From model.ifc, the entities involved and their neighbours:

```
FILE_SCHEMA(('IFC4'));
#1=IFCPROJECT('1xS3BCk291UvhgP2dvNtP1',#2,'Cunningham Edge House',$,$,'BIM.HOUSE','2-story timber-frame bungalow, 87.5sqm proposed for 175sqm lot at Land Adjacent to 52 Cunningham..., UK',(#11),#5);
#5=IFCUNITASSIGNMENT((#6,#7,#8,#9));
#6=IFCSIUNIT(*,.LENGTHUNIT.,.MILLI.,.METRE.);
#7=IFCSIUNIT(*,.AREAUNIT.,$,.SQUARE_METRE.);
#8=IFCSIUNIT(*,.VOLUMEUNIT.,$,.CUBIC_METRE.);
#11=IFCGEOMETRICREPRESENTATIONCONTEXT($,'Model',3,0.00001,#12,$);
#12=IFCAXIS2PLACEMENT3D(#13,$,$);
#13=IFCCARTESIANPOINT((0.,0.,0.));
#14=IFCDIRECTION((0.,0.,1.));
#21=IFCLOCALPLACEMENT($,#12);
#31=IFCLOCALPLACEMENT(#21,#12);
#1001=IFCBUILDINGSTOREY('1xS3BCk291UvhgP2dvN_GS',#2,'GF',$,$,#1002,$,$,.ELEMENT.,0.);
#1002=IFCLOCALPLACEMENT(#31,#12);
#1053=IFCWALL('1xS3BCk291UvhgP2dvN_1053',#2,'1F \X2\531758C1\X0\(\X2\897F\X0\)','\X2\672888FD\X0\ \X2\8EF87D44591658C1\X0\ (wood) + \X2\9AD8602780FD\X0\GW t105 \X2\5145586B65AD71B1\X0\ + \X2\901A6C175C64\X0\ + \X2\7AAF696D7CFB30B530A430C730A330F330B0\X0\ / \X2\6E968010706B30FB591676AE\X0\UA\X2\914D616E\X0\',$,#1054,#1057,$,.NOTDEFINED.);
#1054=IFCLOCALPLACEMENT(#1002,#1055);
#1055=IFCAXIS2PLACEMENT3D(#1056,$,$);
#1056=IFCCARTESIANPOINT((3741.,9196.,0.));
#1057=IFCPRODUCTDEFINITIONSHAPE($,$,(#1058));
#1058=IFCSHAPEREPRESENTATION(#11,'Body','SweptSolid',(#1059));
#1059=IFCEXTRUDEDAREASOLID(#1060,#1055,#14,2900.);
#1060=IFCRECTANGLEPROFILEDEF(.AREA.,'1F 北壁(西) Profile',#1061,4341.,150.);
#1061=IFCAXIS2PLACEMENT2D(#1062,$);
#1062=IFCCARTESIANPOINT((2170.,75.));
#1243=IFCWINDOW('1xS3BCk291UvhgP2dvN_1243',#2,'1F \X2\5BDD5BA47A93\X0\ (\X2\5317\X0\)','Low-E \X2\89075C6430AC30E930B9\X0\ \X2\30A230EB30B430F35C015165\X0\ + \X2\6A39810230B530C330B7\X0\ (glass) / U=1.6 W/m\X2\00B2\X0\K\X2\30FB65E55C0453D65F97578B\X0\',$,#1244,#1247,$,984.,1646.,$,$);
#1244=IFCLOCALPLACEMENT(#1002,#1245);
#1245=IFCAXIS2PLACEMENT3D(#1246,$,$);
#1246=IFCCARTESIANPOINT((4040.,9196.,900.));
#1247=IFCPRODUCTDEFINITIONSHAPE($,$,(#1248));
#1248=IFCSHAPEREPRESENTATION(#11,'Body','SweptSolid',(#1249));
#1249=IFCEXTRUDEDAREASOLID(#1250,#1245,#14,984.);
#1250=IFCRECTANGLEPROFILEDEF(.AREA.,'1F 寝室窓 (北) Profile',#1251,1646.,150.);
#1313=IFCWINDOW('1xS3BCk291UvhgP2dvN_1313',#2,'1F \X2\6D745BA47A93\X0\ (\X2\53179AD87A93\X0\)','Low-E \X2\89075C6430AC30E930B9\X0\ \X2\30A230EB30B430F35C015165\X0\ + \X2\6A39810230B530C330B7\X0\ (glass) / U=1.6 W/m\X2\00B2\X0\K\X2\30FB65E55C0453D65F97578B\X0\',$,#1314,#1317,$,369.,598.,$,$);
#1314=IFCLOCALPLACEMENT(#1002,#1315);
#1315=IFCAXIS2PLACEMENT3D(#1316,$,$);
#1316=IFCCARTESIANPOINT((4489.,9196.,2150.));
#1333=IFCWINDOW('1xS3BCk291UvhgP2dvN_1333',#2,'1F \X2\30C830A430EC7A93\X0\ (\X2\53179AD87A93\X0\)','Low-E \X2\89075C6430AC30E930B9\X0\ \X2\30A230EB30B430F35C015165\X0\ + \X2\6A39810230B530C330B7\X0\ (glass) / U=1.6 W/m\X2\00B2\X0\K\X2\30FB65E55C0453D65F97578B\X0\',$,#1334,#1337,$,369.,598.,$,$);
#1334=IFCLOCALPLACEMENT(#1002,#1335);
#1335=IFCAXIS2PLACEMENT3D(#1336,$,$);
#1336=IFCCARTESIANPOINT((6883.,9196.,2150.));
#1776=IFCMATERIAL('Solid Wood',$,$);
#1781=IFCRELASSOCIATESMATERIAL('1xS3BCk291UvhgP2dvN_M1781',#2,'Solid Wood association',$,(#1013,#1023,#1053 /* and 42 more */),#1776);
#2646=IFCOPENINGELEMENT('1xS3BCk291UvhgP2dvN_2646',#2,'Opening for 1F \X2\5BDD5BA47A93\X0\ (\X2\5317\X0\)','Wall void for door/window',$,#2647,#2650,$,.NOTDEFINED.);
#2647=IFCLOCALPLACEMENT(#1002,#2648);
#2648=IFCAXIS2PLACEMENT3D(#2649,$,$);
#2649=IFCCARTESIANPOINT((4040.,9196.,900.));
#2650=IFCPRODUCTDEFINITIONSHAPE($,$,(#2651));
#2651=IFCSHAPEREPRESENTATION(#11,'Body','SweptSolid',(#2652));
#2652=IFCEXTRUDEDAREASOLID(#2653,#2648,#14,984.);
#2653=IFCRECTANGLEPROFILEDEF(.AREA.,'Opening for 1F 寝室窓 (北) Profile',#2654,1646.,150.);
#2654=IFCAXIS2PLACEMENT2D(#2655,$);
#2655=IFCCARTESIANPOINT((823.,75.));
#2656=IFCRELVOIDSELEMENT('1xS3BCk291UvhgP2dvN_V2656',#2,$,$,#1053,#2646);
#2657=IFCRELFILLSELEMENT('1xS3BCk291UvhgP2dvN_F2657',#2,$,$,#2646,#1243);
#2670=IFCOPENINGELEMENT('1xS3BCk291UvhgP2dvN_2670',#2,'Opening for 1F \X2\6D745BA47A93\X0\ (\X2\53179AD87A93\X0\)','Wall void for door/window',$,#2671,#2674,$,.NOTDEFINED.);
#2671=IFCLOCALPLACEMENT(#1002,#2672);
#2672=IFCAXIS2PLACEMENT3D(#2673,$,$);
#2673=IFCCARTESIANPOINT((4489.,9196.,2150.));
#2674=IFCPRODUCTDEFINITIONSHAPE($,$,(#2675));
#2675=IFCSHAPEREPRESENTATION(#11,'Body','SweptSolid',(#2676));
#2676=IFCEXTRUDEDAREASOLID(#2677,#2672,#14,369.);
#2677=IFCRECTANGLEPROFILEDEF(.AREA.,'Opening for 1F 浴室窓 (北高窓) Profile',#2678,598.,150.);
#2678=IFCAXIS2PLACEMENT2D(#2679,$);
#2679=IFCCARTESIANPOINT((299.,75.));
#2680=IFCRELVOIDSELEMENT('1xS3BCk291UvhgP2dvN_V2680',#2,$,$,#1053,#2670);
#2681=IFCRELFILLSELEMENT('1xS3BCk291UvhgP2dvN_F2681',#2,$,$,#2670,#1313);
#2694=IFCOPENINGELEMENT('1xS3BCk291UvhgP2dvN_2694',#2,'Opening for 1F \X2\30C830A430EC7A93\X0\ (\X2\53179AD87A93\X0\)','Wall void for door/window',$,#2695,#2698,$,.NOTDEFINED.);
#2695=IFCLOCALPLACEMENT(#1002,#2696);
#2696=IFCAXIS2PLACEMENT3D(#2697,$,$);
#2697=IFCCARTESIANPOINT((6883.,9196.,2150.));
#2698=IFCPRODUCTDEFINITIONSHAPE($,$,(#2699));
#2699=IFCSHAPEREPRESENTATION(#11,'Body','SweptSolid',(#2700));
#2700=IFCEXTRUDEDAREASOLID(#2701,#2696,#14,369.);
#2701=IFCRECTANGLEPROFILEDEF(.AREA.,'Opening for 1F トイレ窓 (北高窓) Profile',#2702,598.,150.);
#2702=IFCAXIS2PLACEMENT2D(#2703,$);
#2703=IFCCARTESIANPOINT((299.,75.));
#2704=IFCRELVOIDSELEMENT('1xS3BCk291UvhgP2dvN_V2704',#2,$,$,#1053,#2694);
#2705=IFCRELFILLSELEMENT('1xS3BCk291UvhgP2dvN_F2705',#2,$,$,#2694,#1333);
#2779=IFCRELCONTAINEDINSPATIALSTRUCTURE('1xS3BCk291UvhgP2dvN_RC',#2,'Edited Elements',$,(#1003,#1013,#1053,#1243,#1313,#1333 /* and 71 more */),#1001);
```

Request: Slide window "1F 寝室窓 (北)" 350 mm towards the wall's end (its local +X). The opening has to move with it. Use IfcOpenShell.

```python
import ifcopenshell
import ifcopenshell.api.geometry
import ifcopenshell.util.placement

model = ifcopenshell.open("model.ifc")

window = model.by_guid("1xS3BCk291UvhgP2dvN_1243")
opening = window.FillsVoids[0].RelatingOpeningElement
wall = opening.VoidsElements[0].RelatingBuildingElement

wall_matrix = ifcopenshell.util.placement.get_local_placement(wall.ObjectPlacement)
shift = wall_matrix[:3, 0] * 350.0
before = ifcopenshell.util.placement.get_local_placement(window.ObjectPlacement)[:3, 3].copy()

# The window is not placed relative to its opening, so move both.
for product in (opening, window):
    matrix = ifcopenshell.util.placement.get_local_placement(product.ObjectPlacement)
    matrix[:3, 3] += shift
    ifcopenshell.api.geometry.edit_object_placement(model, product=product, matrix=matrix, is_si=False)

after = ifcopenshell.util.placement.get_local_placement(window.ObjectPlacement)[:3, 3]
print("window moved by", (after - before).round(3) + 0.0)

model.write("model_rev.ifc")
```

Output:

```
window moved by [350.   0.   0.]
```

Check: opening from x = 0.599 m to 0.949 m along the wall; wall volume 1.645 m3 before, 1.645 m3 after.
